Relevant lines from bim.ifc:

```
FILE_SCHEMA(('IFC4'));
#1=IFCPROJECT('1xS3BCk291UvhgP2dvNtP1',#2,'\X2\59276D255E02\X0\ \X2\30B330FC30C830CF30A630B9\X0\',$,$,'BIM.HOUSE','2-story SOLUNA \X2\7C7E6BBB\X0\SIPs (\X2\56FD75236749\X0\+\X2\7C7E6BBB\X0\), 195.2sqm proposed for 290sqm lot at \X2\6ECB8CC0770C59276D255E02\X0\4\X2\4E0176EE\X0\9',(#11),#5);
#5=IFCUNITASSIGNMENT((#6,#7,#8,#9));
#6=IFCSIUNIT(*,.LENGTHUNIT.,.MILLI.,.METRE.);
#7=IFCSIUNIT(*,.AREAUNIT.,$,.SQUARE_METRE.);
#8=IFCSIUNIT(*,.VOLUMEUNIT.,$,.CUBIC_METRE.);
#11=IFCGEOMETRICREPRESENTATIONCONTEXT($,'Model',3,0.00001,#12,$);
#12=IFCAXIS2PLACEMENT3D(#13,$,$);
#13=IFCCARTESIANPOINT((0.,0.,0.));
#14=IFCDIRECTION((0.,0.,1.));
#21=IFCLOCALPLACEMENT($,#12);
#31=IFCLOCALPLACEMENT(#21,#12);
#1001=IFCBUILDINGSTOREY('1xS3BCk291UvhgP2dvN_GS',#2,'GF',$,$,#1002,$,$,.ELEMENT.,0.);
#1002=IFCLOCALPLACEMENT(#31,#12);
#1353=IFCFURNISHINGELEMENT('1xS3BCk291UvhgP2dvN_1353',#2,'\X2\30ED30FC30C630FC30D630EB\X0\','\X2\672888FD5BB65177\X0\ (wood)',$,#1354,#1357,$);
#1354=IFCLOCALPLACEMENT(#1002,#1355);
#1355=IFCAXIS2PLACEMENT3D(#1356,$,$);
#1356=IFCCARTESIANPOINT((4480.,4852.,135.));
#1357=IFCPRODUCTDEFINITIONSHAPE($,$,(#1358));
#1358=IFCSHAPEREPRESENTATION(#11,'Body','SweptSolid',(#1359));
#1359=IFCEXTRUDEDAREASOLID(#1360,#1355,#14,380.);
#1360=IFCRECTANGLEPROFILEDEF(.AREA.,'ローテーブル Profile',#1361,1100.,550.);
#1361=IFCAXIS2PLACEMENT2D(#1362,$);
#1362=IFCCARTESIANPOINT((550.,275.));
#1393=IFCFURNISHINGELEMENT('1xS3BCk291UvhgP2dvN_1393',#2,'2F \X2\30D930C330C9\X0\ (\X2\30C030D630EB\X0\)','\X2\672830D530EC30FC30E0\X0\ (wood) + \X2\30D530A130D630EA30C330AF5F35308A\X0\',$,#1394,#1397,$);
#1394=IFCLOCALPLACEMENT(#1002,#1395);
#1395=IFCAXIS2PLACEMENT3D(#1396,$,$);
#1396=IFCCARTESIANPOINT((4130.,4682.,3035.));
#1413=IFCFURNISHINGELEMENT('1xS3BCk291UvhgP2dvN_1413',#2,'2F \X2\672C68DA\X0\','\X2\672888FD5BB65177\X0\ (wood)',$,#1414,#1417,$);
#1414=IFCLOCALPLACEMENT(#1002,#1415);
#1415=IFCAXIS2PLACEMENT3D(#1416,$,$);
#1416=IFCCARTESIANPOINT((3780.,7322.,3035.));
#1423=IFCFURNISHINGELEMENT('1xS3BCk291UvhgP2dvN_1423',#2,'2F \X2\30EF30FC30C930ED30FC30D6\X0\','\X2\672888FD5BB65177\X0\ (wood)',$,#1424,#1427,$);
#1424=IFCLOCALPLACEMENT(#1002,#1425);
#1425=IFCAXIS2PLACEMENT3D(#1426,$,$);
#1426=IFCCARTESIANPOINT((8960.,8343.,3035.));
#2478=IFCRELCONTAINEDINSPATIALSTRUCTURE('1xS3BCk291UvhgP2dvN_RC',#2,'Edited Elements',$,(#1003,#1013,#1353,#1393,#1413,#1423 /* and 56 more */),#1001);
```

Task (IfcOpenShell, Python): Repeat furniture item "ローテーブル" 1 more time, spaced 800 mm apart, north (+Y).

```python
import numpy as np
import ifcopenshell
import ifcopenshell.api.geometry
import ifcopenshell.api.root
import ifcopenshell.util.element
import ifcopenshell.util.placement
import ifcopenshell.util.unit

model = ifcopenshell.open("bim.ifc")
unit_scale = ifcopenshell.util.unit.calculate_unit_scale(model)


def reuse_history(source, copy):
    """copy_class also copies each property set's owner history, people and application; keep the originals."""
    for rel in copy.IsDefinedBy:
        if rel.is_a("IfcRelDefinesByProperties") and (history := rel.RelatingPropertyDefinition.OwnerHistory):
            rel.RelatingPropertyDefinition.OwnerHistory = source.OwnerHistory
            ifcopenshell.util.element.remove_deep2(model, history)


source = model.by_id(1353)
base = ifcopenshell.util.placement.get_local_placement(source.ObjectPlacement)
step = np.array([0.0, 1.0, 0.0]) * 0.8 / unit_scale

for i in range(1, 2):
    copy = ifcopenshell.api.root.copy_class(model, product=source)
    copy.Representation = ifcopenshell.util.element.copy_deep(
        model, source.Representation, exclude=["IfcGeometricRepresentationContext", "IfcRepresentationMap"]
    )
    reuse_history(source, copy)
    matrix = base.copy()
    matrix[:3, 3] += i * step
    print("added at", matrix[:3, 3].round(3) + 0.0)
    ifcopenshell.api.geometry.edit_object_placement(model, product=copy, matrix=matrix, is_si=False)

model.write("bim_v2.ifc")
```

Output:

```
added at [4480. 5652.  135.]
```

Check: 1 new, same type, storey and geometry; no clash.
